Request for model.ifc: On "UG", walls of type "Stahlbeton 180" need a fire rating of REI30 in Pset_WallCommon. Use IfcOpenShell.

First a look at what the model holds.

```python
import ifcopenshell
import ifcopenshell.util.element

model = ifcopenshell.open("model.ifc")
print(model.schema)
storey = next(s for s in model.by_type("IfcBuildingStorey") if s.Name == "UG")
walls = [e for e in ifcopenshell.util.element.get_decomposition(storey) if e.is_a("IfcWall")]
seen = {}
for e in walls:
    element_type = ifcopenshell.util.element.get_type(e)
    key = (element_type.Name if element_type != e and element_type else None, ifcopenshell.util.element.get_pset(e, "Pset_WallCommon", "FireRating"))
    seen[key] = seen.get(key, 0) + 1
for (name, value), count in sorted(seen.items(), key=str):
    print(count, "x", name, "|", value)
```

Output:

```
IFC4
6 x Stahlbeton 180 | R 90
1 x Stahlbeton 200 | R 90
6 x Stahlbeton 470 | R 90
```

```python
import ifcopenshell
import ifcopenshell.api.pset
import ifcopenshell.util.element

model = ifcopenshell.open("model.ifc")

storey = next(s for s in model.by_type("IfcBuildingStorey") if s.Name == "UG")
walls = [e for e in ifcopenshell.util.element.get_decomposition(storey) if e.is_a("IfcWall")]

count = 0
for e in walls:
    element_type = ifcopenshell.util.element.get_type(e)
    if element_type in (None, e) or element_type.Name != "Stahlbeton 180":
        continue
    # add_pset returns the element's existing set when there is one.
    pset = ifcopenshell.api.pset.add_pset(model, product=e, name="Pset_WallCommon")
    ifcopenshell.api.pset.edit_pset(model, pset=pset, properties={"FireRating": "REI30"})
    count += 1

print(count, "walls updated")

model.write("model_updated.ifc")
```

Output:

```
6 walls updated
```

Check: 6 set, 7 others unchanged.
